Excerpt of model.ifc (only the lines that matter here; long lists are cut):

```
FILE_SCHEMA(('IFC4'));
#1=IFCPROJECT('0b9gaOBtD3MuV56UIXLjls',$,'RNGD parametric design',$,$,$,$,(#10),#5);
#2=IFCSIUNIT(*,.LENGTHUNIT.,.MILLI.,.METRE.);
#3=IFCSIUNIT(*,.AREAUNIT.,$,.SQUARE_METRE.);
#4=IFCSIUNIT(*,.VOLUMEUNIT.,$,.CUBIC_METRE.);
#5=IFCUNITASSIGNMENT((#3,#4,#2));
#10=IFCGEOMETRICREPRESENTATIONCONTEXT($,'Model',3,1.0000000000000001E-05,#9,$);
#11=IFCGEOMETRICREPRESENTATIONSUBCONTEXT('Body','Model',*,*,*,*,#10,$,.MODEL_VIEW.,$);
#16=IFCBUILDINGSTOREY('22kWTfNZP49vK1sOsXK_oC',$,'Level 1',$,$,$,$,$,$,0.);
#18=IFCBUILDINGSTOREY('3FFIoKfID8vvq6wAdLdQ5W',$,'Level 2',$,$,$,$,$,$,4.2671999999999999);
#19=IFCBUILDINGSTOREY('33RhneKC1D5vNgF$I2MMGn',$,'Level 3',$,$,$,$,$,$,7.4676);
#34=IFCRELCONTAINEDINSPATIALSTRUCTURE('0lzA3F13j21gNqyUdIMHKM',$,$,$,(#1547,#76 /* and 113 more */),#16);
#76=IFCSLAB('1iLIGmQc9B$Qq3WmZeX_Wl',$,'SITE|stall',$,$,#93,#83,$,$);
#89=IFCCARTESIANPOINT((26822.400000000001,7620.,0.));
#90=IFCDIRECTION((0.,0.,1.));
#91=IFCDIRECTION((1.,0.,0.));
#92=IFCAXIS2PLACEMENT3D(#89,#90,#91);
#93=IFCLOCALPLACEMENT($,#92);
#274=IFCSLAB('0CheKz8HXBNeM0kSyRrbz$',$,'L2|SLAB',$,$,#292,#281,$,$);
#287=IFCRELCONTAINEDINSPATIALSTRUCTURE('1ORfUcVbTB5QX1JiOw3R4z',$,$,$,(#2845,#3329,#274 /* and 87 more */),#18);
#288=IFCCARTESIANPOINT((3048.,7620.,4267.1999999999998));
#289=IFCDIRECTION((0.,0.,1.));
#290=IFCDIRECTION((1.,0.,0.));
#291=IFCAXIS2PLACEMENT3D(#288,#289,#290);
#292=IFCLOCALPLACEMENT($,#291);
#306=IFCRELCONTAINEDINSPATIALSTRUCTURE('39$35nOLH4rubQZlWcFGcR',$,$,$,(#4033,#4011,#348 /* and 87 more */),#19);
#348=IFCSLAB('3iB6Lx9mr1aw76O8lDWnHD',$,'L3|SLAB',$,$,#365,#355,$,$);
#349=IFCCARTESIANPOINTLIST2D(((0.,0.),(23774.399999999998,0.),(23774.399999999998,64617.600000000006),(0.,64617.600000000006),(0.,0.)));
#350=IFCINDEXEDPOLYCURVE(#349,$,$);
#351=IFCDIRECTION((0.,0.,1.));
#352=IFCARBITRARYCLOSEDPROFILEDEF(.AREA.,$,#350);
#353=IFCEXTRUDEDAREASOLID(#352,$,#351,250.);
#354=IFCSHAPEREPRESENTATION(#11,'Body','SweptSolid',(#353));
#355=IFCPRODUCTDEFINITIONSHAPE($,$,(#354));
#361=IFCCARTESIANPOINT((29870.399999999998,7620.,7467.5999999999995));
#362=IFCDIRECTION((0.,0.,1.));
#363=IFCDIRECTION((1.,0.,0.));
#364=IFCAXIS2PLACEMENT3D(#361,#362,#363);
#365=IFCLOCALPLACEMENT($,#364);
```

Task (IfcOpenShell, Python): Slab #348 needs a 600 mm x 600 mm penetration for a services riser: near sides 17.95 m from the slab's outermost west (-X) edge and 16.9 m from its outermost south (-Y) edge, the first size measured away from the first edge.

```python
import numpy as np
import ifcopenshell
import ifcopenshell.api.feature
import ifcopenshell.api.geometry
import ifcopenshell.api.root
import ifcopenshell.geom
import ifcopenshell.util.placement
import ifcopenshell.util.representation
import ifcopenshell.util.shape
import ifcopenshell.util.unit

model = ifcopenshell.open("model.ifc")
unit_scale = ifcopenshell.util.unit.calculate_unit_scale(model)
settings = ifcopenshell.geom.settings()


def volume(element):
    """Net volume in cubic metres, openings subtracted."""
    shape = ifcopenshell.geom.create_shape(settings, element)
    return ifcopenshell.util.shape.get_volume(shape.geometry)


slab = model.by_guid("3iB6Lx9mr1aw76O8lDWnHD")
before = volume(slab)

# Extent in the slab's own axes, in metres. The edges named are its -X and -Y sides.
slab_shape = ifcopenshell.geom.create_shape(settings, slab)
vertices = ifcopenshell.util.shape.get_vertices(slab_shape.geometry)
x_min, y_min, bottom = vertices.min(axis=0)
top = vertices[:, 2].max()

opening = ifcopenshell.api.root.create_entity(model, ifc_class="IfcOpeningElement", name="Services riser opening", predefined_type="OPENING")
context = ifcopenshell.util.representation.get_context(model, "Model", "Body", "MODEL_VIEW")
width, depth = 0.6, 0.6
outline = [(0.0, 0.0), (width, 0.0), (width, depth), (0.0, depth), (0.0, 0.0)]
# Overshoot both faces by 50 mm so the cut is clean.
shape = ifcopenshell.api.geometry.add_slab_representation(
    model, context=context, depth=top - bottom + 0.1, polyline=outline
)
ifcopenshell.api.geometry.assign_representation(model, product=opening, representation=shape)

matrix = ifcopenshell.util.placement.get_local_placement(slab.ObjectPlacement)
matrix[:, 3] = matrix @ np.append(np.array([x_min + 17.95, y_min + 16.9, bottom - 0.05]) / unit_scale, 1.0)
ifcopenshell.api.geometry.edit_object_placement(model, product=opening, matrix=matrix, is_si=False)
ifcopenshell.api.feature.add_feature(model, feature=opening, element=slab)

after = volume(slab)

print(f"slab volume {before:.3f} -> {after:.3f} m3")

model.write("model_v2.ifc")
```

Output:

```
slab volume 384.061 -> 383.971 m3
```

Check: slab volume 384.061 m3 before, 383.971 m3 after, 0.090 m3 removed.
